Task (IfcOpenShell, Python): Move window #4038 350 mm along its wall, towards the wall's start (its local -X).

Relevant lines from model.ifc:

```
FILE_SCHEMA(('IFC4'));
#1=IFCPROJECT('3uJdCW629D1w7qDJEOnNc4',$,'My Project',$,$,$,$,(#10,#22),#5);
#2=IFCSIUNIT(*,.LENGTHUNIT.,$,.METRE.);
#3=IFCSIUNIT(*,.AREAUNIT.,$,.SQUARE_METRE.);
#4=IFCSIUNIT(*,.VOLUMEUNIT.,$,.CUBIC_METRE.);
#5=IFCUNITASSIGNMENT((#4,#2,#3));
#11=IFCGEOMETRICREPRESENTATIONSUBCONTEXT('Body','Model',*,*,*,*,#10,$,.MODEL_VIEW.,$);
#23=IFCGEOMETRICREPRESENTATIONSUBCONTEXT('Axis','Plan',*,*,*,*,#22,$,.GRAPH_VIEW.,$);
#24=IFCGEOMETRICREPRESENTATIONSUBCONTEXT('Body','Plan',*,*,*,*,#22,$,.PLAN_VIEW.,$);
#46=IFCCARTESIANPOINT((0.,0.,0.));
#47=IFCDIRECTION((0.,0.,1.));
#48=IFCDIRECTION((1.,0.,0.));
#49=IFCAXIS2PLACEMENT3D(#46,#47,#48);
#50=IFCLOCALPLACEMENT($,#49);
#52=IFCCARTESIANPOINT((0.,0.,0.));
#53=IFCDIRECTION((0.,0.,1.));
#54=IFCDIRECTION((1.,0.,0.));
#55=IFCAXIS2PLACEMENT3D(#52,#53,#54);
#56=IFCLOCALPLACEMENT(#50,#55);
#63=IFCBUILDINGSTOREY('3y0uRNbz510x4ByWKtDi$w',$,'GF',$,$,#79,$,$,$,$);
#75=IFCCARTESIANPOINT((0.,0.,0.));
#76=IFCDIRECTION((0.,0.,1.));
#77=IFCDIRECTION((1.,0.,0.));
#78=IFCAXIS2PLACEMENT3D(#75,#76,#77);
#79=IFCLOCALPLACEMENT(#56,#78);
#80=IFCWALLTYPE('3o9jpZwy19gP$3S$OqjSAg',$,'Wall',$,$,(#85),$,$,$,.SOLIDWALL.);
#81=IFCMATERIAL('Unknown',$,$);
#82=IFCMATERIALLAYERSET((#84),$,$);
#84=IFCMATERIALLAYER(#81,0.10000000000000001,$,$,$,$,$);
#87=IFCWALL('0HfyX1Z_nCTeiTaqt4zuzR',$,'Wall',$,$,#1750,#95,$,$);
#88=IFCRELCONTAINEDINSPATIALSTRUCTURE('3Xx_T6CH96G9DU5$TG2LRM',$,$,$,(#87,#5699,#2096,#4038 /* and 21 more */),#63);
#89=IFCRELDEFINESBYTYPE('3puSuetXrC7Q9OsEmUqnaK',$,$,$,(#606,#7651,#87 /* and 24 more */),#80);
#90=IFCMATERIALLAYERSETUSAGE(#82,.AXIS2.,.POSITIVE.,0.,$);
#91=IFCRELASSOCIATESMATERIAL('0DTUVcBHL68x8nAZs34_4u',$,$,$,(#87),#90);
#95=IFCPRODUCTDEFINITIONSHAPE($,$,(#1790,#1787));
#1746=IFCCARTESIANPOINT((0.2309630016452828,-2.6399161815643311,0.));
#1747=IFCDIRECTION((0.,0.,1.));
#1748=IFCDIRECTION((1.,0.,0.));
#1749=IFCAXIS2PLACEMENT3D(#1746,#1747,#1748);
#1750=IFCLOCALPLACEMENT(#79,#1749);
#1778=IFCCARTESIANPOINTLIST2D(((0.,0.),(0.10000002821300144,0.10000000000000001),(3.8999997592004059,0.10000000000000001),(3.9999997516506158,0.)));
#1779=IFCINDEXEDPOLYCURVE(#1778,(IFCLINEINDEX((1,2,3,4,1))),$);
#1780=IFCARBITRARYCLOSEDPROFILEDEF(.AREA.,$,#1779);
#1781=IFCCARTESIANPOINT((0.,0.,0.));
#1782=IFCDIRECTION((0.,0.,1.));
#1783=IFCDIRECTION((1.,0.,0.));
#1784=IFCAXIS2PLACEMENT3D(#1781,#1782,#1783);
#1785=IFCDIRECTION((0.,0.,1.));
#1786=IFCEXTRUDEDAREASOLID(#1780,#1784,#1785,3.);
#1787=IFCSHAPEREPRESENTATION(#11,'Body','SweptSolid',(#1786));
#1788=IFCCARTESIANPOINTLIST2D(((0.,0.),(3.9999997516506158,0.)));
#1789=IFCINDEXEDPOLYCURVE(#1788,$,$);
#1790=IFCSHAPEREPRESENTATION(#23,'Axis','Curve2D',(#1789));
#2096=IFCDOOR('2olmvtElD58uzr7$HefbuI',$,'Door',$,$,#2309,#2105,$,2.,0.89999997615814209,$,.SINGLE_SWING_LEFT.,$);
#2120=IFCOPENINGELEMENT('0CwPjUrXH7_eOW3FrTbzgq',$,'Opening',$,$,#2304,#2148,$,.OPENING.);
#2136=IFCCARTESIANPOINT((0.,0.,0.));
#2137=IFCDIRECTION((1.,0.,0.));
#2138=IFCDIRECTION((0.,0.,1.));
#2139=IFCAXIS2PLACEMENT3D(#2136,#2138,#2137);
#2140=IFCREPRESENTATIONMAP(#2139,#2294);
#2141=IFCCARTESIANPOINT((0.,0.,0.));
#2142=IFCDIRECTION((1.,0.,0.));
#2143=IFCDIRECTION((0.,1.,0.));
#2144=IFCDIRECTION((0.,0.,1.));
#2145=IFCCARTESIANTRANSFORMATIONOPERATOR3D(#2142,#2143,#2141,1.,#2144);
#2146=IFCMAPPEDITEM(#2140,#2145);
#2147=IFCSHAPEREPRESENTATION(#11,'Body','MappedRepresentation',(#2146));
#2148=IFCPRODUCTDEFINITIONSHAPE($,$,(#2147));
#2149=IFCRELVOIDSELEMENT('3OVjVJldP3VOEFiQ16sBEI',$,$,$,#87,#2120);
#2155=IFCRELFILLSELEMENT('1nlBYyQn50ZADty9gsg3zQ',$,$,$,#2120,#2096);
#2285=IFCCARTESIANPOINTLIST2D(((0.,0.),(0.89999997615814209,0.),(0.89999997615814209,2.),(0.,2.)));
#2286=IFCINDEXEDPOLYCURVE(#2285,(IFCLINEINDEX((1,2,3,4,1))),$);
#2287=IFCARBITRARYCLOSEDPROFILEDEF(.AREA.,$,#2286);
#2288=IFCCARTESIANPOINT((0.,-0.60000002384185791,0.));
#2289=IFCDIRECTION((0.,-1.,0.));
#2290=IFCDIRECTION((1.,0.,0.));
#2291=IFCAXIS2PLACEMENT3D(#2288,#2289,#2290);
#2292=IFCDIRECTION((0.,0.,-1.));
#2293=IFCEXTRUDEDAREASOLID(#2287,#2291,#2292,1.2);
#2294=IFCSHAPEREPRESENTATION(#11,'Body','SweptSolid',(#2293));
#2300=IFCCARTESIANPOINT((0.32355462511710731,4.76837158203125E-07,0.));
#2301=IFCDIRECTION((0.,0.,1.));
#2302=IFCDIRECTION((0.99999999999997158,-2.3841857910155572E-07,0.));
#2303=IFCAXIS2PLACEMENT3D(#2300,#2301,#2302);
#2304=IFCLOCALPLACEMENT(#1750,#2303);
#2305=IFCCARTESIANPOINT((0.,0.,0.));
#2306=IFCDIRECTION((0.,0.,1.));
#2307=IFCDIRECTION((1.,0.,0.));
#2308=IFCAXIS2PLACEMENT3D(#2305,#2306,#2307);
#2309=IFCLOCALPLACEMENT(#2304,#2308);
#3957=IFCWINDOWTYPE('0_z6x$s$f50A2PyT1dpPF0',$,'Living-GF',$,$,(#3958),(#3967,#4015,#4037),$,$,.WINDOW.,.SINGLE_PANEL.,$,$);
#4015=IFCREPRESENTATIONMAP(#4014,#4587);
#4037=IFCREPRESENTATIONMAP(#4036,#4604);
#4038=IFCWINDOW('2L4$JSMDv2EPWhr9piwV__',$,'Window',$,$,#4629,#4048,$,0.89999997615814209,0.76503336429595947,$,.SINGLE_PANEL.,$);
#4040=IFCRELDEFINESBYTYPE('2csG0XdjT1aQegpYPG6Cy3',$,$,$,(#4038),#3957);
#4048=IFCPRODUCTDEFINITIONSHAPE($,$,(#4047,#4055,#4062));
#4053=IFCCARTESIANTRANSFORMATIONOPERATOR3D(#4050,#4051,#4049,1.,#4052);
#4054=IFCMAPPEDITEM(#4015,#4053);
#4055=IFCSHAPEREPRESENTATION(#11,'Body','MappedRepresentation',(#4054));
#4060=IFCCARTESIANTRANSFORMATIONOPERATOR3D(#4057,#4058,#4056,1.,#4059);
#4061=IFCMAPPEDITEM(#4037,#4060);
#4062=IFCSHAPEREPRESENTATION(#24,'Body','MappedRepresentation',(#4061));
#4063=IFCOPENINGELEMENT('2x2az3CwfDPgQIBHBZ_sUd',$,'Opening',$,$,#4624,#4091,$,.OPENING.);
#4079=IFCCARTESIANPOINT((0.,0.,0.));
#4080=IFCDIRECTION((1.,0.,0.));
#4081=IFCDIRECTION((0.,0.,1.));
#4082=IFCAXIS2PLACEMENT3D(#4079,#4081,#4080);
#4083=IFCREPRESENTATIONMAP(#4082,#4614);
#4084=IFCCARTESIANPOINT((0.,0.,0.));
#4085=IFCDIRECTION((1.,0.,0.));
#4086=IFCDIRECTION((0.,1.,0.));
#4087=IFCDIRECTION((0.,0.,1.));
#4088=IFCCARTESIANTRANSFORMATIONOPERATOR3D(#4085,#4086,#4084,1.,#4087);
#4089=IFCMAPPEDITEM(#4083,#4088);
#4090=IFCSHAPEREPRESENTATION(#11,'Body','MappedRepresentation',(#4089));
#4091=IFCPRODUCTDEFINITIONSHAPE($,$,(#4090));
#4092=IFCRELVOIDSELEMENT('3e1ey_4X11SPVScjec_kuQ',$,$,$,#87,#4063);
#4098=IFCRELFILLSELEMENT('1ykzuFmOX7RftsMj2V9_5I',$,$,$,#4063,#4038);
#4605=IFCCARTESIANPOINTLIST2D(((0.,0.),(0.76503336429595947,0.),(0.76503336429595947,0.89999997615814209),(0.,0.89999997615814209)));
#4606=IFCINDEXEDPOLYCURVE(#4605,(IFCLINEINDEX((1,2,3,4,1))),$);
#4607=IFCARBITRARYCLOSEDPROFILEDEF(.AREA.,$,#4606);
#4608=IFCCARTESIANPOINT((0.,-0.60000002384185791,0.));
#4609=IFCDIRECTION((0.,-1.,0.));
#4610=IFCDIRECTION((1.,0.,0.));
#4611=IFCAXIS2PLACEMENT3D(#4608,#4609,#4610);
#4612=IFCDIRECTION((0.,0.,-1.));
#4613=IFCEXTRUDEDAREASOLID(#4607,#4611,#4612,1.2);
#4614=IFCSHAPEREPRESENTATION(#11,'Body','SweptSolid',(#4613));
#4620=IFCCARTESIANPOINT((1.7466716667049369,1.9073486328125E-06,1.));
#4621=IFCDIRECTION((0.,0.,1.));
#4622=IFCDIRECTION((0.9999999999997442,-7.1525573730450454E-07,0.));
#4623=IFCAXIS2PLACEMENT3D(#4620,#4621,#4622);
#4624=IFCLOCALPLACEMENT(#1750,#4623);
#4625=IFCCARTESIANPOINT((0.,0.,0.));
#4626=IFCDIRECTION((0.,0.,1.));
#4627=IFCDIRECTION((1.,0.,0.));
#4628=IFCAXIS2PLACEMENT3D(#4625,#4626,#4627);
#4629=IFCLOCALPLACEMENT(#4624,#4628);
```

```python
import ifcopenshell
import ifcopenshell.api.geometry
import ifcopenshell.util.placement
import ifcopenshell.util.unit

model = ifcopenshell.open("model.ifc")
unit_scale = ifcopenshell.util.unit.calculate_unit_scale(model)

window = model.by_guid("2L4$JSMDv2EPWhr9piwV__")
opening = window.FillsVoids[0].RelatingOpeningElement
wall = opening.VoidsElements[0].RelatingBuildingElement

wall_matrix = ifcopenshell.util.placement.get_local_placement(wall.ObjectPlacement)
shift = wall_matrix[:3, 0] * -0.35 / unit_scale
before = ifcopenshell.util.placement.get_local_placement(window.ObjectPlacement)[:3, 3].copy()

# The window is placed relative to its opening, so it follows when the opening moves.
matrix = ifcopenshell.util.placement.get_local_placement(opening.ObjectPlacement)
matrix[:3, 3] += shift
ifcopenshell.api.geometry.edit_object_placement(
    model, product=opening, matrix=matrix, is_si=False, should_transform_children=True
)

after = ifcopenshell.util.placement.get_local_placement(window.ObjectPlacement)[:3, 3]
print("window moved by", (after - before).round(3) + 0.0)

model.write("model-out.ifc")
```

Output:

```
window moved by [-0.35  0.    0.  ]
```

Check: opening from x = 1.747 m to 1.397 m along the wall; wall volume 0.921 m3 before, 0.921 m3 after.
